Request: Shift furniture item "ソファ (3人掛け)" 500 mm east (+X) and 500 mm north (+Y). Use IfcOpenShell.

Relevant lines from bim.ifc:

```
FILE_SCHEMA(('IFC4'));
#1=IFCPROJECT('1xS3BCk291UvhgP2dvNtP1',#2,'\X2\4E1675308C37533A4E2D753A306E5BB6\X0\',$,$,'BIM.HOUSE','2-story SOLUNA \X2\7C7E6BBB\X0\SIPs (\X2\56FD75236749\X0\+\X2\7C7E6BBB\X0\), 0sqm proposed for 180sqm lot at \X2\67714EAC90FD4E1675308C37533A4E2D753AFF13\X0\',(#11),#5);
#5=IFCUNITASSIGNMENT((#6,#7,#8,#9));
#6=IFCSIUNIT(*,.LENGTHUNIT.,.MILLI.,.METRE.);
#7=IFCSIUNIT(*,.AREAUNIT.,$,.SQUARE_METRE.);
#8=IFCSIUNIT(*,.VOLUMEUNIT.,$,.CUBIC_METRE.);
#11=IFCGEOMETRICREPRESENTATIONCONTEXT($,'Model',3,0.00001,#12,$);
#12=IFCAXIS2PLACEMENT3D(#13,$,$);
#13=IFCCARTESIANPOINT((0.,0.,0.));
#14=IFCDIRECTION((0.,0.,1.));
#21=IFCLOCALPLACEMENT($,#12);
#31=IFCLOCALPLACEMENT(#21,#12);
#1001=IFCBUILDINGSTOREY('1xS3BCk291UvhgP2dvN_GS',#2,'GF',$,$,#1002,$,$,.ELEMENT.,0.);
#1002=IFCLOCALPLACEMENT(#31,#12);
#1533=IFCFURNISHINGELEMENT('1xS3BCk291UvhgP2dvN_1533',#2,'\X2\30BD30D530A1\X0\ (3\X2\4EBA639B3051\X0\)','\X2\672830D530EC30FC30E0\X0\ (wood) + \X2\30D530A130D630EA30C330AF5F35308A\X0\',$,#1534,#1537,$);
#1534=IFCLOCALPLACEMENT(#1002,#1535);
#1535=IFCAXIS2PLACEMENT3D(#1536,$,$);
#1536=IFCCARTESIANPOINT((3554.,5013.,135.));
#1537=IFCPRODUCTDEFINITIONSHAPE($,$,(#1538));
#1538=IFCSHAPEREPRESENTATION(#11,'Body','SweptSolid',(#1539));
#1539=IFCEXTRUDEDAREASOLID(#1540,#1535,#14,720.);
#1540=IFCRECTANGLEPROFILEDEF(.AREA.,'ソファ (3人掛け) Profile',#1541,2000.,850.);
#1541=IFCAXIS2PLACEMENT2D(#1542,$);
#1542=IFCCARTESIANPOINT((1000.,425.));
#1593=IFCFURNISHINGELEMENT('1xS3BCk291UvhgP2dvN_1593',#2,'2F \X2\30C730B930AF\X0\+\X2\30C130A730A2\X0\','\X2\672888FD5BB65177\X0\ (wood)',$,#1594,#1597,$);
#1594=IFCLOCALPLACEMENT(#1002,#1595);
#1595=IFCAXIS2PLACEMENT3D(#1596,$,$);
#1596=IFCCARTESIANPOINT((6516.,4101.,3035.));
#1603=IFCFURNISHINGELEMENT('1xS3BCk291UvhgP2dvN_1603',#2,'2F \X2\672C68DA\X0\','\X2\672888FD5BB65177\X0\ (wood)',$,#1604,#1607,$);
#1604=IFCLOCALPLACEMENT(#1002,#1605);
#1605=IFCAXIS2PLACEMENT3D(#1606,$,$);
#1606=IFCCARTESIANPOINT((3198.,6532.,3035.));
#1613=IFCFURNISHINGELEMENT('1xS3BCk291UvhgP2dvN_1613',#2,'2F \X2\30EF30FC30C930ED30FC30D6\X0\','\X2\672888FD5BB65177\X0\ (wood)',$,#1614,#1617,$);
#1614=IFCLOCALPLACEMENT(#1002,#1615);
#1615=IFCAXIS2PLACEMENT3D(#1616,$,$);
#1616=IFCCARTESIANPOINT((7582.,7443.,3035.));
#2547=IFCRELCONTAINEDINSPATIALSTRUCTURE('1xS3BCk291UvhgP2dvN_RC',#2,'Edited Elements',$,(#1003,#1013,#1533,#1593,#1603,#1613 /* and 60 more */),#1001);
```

```python
import ifcopenshell
import ifcopenshell.api.geometry
import ifcopenshell.util.placement
import ifcopenshell.util.unit

model = ifcopenshell.open("bim.ifc")
unit_scale = ifcopenshell.util.unit.calculate_unit_scale(model)

item = model.by_guid("1xS3BCk291UvhgP2dvN_1533")
matrix = ifcopenshell.util.placement.get_local_placement(item.ObjectPlacement)
matrix[0, 3] += 0.5 / unit_scale
matrix[1, 3] += 0.5 / unit_scale
ifcopenshell.api.geometry.edit_object_placement(model, product=item, matrix=matrix, is_si=False)

print(ifcopenshell.util.placement.get_local_placement(item.ObjectPlacement).round(3) + 0.0)

model.write("bim-out.ifc")
```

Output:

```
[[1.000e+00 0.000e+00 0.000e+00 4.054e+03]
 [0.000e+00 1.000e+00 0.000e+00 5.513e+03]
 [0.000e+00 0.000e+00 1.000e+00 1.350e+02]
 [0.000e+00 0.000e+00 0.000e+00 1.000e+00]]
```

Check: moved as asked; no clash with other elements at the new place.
